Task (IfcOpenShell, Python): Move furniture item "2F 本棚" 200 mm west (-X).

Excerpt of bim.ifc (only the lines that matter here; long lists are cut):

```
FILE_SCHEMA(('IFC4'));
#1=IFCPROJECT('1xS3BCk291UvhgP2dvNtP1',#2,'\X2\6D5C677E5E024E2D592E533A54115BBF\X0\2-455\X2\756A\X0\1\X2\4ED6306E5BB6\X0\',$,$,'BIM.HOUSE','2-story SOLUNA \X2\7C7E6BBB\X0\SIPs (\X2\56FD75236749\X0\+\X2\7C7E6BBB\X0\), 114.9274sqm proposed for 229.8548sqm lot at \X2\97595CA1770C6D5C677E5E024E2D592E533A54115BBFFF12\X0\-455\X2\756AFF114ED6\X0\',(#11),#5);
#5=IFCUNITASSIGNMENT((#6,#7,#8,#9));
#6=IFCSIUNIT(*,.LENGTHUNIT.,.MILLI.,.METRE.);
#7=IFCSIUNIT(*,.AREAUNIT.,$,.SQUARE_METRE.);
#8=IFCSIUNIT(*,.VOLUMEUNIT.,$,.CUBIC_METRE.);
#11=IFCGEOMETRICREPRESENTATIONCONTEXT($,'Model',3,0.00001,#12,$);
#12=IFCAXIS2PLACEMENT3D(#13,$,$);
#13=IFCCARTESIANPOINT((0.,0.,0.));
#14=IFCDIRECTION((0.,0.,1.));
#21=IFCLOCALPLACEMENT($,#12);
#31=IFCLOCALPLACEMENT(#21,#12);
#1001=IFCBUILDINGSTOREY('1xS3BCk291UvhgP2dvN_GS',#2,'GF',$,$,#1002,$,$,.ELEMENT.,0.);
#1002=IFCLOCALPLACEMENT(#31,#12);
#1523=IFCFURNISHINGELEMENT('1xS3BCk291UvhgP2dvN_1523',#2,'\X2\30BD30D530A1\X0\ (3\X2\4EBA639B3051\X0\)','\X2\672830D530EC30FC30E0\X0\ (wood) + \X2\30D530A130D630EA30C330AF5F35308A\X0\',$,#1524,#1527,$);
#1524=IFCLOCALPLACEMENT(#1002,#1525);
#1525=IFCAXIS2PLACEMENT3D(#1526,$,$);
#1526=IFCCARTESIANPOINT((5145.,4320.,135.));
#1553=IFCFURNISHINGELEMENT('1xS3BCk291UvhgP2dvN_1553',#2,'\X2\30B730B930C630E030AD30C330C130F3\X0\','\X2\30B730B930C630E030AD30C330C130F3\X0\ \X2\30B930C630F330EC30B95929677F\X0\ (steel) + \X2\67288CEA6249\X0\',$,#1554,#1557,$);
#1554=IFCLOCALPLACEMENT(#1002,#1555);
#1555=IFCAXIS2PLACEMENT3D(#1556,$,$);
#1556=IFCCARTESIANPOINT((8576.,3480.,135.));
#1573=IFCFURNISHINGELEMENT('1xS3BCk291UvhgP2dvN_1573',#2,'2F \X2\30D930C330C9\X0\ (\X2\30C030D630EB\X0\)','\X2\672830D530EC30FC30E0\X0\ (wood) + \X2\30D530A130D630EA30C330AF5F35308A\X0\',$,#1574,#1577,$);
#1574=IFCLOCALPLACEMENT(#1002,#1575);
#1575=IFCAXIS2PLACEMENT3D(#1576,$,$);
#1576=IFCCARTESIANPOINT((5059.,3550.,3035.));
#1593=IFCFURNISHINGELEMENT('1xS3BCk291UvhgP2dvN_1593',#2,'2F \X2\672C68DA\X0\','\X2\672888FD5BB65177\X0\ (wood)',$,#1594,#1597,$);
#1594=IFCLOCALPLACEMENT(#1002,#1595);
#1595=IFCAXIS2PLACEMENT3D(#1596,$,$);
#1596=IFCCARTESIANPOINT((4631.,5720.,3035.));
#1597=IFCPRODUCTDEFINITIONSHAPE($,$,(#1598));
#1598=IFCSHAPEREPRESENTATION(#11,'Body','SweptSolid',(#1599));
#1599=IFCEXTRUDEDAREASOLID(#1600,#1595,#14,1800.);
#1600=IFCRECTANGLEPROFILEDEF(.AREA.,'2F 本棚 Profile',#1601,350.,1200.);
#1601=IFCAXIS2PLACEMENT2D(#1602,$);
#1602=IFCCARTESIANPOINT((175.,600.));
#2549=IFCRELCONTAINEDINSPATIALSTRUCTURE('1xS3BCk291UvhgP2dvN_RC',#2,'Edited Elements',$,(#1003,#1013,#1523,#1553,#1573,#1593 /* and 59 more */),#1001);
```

```python
import ifcopenshell
import ifcopenshell.api.geometry
import ifcopenshell.util.placement
import ifcopenshell.util.unit

model = ifcopenshell.open("bim.ifc")
unit_scale = ifcopenshell.util.unit.calculate_unit_scale(model)

item = model.by_guid("1xS3BCk291UvhgP2dvN_1593")
matrix = ifcopenshell.util.placement.get_local_placement(item.ObjectPlacement)
matrix[0, 3] -= 0.2 / unit_scale
ifcopenshell.api.geometry.edit_object_placement(model, product=item, matrix=matrix, is_si=False)

print(ifcopenshell.util.placement.get_local_placement(item.ObjectPlacement).round(3) + 0.0)

model.write("bim-out.ifc")
```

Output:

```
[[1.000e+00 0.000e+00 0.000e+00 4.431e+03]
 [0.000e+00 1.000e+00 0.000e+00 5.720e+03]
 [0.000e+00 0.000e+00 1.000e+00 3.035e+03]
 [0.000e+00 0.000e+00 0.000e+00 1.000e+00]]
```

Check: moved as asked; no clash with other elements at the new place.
